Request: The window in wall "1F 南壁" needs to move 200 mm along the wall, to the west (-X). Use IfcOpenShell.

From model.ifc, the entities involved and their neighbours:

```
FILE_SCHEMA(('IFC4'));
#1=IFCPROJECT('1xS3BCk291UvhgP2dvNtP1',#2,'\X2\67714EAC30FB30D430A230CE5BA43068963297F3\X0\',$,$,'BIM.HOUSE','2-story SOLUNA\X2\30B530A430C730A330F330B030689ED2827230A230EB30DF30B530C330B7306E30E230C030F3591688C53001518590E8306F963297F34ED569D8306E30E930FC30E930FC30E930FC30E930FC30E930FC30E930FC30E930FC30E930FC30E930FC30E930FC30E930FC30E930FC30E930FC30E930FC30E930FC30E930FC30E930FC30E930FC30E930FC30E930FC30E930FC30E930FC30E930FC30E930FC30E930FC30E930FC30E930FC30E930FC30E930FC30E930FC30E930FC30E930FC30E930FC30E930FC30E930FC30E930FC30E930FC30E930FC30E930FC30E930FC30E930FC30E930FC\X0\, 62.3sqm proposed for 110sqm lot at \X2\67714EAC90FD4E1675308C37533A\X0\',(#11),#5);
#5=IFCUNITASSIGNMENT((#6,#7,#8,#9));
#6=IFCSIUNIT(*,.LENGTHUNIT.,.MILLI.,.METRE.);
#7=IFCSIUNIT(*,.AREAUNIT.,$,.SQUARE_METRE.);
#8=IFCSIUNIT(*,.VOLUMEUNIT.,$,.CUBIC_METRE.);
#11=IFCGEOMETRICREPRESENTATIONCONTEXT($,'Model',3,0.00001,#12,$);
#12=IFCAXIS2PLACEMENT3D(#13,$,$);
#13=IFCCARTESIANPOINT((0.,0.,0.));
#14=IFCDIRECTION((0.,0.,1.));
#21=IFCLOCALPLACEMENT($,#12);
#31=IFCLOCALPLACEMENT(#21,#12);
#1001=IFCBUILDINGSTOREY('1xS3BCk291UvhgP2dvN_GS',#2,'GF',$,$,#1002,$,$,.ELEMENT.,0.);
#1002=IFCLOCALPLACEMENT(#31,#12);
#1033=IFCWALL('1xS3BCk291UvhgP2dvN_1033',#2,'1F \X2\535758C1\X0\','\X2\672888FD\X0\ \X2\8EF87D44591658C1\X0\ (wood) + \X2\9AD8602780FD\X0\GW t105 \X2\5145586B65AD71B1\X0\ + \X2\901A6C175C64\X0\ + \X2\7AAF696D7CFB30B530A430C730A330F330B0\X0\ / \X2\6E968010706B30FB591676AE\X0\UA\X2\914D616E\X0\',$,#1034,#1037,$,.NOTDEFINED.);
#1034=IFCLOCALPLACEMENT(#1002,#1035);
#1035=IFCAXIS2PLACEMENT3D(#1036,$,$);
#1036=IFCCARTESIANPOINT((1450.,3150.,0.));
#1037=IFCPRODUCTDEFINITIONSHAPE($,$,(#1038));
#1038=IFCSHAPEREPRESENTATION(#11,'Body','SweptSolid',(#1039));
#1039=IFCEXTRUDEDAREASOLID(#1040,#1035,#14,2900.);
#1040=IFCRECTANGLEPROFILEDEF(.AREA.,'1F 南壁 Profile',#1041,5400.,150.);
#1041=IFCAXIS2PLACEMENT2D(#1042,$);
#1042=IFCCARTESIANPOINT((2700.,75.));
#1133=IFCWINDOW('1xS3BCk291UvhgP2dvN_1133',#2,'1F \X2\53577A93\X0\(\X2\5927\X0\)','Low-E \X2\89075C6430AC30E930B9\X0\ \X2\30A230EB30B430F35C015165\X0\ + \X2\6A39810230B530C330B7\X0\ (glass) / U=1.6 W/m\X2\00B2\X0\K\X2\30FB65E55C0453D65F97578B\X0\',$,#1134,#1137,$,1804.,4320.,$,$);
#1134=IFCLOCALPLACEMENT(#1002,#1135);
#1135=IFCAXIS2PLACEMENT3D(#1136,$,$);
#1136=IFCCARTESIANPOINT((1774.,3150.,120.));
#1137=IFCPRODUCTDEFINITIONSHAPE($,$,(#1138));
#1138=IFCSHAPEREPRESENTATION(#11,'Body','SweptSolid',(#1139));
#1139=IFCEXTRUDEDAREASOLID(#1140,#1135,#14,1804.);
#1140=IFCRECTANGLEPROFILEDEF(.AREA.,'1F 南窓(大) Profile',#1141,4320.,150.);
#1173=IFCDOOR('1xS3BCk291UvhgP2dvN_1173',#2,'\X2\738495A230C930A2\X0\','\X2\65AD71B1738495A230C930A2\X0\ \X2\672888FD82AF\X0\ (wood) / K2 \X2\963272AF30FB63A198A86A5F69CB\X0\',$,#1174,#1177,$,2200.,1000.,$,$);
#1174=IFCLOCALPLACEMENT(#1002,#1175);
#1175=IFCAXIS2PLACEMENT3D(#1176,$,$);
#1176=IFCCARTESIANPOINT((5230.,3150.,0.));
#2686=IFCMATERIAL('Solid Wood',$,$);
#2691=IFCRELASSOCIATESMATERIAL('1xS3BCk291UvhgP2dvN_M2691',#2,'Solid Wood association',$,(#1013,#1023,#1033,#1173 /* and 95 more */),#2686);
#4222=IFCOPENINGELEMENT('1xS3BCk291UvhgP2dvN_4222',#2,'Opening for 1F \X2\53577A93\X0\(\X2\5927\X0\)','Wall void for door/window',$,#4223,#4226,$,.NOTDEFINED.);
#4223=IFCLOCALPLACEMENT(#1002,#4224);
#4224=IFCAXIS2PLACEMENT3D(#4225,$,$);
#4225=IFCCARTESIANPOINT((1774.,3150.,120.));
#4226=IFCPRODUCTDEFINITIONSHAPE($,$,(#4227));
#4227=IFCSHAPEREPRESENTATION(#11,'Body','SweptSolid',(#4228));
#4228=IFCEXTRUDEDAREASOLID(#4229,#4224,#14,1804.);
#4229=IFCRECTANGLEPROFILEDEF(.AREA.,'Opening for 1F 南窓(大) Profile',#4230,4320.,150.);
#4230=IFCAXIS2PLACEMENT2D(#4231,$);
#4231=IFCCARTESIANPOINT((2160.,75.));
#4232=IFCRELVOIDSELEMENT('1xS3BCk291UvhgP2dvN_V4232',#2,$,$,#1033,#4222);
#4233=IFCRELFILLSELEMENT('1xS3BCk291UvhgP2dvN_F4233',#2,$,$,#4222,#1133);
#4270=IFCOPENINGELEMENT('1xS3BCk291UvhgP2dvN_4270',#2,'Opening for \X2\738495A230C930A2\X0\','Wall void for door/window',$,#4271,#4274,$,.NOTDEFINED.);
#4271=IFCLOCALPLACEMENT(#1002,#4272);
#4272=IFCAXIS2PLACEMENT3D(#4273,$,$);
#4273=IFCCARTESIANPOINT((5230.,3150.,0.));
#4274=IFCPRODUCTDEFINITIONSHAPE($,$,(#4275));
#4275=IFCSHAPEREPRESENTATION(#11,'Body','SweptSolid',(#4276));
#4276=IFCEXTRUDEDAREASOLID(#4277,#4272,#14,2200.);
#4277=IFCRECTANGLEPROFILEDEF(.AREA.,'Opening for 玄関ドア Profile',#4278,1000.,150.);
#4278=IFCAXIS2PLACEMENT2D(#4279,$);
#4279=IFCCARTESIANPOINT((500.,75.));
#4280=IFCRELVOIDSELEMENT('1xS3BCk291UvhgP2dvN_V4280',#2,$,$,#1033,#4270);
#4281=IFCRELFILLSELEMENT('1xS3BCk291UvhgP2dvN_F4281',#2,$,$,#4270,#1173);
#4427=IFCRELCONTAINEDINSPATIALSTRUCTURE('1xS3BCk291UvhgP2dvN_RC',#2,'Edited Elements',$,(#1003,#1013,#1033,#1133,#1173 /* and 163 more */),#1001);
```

```python
import ifcopenshell
import ifcopenshell.api.geometry
import ifcopenshell.util.placement

model = ifcopenshell.open("model.ifc")

window = model.by_id(1133)
opening = window.FillsVoids[0].RelatingOpeningElement
wall = opening.VoidsElements[0].RelatingBuildingElement

wall_matrix = ifcopenshell.util.placement.get_local_placement(wall.ObjectPlacement)
shift = wall_matrix[:3, 0] * -200.0
before = ifcopenshell.util.placement.get_local_placement(window.ObjectPlacement)[:3, 3].copy()

# The window is not placed relative to its opening, so move both.
for product in (opening, window):
    matrix = ifcopenshell.util.placement.get_local_placement(product.ObjectPlacement)
    matrix[:3, 3] += shift
    ifcopenshell.api.geometry.edit_object_placement(model, product=product, matrix=matrix, is_si=False)

after = ifcopenshell.util.placement.get_local_placement(window.ObjectPlacement)[:3, 3]
print("window moved by", (after - before).round(3) + 0.0)

model.write("model_v2.ifc")
```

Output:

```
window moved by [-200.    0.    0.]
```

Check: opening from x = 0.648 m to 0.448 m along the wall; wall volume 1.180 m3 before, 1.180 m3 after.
